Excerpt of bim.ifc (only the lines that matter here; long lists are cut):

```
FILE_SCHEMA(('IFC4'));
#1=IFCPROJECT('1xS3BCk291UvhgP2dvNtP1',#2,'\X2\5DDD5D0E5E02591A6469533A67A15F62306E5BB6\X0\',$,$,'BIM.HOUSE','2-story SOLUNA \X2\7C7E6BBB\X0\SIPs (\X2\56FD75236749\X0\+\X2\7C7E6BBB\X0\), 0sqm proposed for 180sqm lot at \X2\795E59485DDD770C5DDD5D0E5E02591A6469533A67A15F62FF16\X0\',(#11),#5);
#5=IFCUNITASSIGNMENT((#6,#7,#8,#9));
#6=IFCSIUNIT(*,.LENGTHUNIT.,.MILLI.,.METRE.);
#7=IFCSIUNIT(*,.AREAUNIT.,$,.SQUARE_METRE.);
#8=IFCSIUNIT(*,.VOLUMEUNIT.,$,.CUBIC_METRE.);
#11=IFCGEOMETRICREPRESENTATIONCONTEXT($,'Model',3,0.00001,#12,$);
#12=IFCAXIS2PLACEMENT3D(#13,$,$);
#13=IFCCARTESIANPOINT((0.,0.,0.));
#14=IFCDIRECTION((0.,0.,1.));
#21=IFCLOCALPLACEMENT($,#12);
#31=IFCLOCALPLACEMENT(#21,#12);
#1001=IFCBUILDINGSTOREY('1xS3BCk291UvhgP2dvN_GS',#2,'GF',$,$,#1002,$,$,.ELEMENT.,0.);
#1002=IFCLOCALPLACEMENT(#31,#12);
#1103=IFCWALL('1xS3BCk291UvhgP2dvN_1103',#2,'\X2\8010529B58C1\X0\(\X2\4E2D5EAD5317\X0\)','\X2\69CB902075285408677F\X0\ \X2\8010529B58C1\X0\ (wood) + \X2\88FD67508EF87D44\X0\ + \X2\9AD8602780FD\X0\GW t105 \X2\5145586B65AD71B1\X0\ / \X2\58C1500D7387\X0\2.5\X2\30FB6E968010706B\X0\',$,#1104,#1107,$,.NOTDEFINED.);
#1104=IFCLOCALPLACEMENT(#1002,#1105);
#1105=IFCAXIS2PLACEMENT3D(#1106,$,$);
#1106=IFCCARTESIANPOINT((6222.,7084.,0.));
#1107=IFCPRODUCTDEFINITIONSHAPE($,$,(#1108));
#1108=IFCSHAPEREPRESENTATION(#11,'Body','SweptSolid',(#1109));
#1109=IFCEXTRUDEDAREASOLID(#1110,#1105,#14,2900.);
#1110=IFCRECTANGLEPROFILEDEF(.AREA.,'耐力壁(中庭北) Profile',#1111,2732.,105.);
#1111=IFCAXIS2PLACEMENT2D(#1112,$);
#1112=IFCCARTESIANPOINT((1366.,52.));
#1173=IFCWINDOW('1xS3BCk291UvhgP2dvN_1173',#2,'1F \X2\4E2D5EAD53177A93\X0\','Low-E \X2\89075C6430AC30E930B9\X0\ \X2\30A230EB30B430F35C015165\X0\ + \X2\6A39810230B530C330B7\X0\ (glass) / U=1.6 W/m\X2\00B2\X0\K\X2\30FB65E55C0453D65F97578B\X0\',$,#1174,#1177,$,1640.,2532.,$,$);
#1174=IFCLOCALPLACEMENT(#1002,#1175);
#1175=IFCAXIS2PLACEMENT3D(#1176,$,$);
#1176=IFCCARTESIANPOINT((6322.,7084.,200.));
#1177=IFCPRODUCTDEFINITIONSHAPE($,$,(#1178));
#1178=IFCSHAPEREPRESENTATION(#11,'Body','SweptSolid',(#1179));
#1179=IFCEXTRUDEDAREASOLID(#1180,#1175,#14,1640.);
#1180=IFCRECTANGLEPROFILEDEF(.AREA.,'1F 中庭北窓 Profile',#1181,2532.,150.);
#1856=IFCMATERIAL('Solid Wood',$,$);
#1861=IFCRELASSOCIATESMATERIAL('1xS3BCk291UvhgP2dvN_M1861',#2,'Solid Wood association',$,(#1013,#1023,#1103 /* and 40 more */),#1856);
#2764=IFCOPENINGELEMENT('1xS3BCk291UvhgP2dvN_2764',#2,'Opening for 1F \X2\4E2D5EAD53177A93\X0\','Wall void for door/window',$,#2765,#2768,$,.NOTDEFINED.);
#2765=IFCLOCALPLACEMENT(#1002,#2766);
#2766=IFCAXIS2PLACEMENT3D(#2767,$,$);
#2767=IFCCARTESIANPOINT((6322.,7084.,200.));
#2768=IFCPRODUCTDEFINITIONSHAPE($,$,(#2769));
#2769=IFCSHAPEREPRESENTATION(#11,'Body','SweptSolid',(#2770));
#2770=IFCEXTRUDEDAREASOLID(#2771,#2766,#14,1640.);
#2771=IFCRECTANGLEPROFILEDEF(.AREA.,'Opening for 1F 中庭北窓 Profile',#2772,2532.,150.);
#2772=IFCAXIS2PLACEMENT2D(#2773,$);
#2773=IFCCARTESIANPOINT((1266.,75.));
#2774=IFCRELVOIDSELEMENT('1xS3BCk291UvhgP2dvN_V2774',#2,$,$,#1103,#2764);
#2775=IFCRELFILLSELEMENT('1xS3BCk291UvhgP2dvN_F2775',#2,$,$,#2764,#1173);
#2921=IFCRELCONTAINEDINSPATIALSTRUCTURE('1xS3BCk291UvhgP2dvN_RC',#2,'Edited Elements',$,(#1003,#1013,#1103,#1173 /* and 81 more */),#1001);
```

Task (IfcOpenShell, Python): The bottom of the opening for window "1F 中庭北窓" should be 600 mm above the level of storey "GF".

```python
import numpy as np
import ifcopenshell
import ifcopenshell.api.geometry
import ifcopenshell.geom
import ifcopenshell.util.element
import ifcopenshell.util.placement
import ifcopenshell.util.shape
import ifcopenshell.util.unit

model = ifcopenshell.open("bim.ifc")
unit_scale = ifcopenshell.util.unit.calculate_unit_scale(model)

window = model.by_guid("1xS3BCk291UvhgP2dvN_1173")
opening = window.FillsVoids[0].RelatingOpeningElement
storey = ifcopenshell.util.element.get_container(window, ifc_class="IfcBuildingStorey")
level = ifcopenshell.util.placement.get_local_placement(storey.ObjectPlacement)[2, 3]

# The opening's origin need not be at the sill, so measure its lowest point.
shape = ifcopenshell.geom.create_shape(ifcopenshell.geom.settings(), opening)
bottom = ifcopenshell.util.shape.get_shape_bottom_elevation(shape, shape.geometry) / unit_scale
dz = level + 600.0 - bottom

shift = np.array([0.0, 0.0, dz])
# The window is not placed relative to its opening, so move both.
for product in (opening, window):
    matrix = ifcopenshell.util.placement.get_local_placement(product.ObjectPlacement)
    matrix[:3, 3] += shift
    ifcopenshell.api.geometry.edit_object_placement(model, product=product, matrix=matrix, is_si=False)

print(f"moved by {dz * unit_scale:+.3f} m")

model.write("bim_updated.ifc")
```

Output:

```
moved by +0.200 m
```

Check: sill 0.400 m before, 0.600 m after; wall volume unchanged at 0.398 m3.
